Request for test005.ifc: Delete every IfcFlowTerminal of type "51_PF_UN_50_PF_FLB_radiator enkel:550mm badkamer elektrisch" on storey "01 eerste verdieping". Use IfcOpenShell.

First a look at what the model holds.

```python
import ifcopenshell
import ifcopenshell.util.element

model = ifcopenshell.open("test005.ifc")
print(model.schema)
storey = next(s for s in model.by_type("IfcBuildingStorey") if s.Name == "01 eerste verdieping")
terminals = [e for e in ifcopenshell.util.element.get_decomposition(storey) if e.is_a("IfcFlowTerminal")]
seen = {}
for e in terminals:
    element_type = ifcopenshell.util.element.get_type(e)
    name = element_type.Name if element_type not in (None, e) else None
    seen[name] = seen.get(name, 0) + 1
for name, count in sorted(seen.items(), key=str):
    print(count, "x", name)
```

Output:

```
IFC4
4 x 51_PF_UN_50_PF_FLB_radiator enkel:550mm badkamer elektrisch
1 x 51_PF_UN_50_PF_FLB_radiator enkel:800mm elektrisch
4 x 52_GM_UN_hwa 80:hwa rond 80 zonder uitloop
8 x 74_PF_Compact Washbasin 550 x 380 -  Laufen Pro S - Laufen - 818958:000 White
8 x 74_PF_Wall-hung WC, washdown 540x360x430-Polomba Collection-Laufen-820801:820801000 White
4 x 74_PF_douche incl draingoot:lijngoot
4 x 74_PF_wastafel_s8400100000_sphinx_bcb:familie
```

```python
import ifcopenshell
import ifcopenshell.api.root
import ifcopenshell.util.element

model = ifcopenshell.open("test005.ifc")

storey = next(s for s in model.by_type("IfcBuildingStorey") if s.Name == "01 eerste verdieping")
terminals = [e for e in ifcopenshell.util.element.get_decomposition(storey) if e.is_a("IfcFlowTerminal")]
targets = [e for e in terminals if (t := ifcopenshell.util.element.get_type(e)) not in (None, e) and t.Name == "51_PF_UN_50_PF_FLB_radiator enkel:550mm badkamer elektrisch"]

for e in targets:
    ifcopenshell.api.root.remove_product(model, product=e)
print(len(targets), "removed")

model.write("test005_edited.ifc")
```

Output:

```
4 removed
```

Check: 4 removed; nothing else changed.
